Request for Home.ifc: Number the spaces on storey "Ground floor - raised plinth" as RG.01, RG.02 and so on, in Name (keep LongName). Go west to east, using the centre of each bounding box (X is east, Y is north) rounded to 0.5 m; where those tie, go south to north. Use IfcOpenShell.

First a look at what the model holds.

```python
import ifcopenshell
import ifcopenshell.util.element
import ifcopenshell.util.placement

model = ifcopenshell.open("Home.ifc")
print(model.schema)
storey = next(s for s in model.by_type("IfcBuildingStorey") if s.Name == "Ground floor - raised plinth")
spaces = [e for e in ifcopenshell.util.element.get_decomposition(storey) if e.is_a("IfcSpace")]
for e in sorted(spaces, key=lambda e: e.id()):
    origin = ifcopenshell.util.placement.get_local_placement(e.ObjectPlacement)[:3, 3]
    print(e.id(), e.Name, e.LongName, origin.round(2) + 0.0, sep=" | ")
```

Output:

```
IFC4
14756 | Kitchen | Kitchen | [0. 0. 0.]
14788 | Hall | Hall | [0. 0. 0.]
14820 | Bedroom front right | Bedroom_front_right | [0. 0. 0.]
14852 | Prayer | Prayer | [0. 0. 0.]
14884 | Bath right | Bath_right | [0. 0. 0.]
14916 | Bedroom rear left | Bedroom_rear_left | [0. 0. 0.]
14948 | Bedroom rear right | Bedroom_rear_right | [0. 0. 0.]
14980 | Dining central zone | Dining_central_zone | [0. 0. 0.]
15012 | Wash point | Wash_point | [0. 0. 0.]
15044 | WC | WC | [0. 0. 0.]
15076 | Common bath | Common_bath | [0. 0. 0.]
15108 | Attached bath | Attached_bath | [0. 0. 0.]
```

```python
import ifcopenshell
import ifcopenshell.geom
import ifcopenshell.util.element
import ifcopenshell.util.shape

model = ifcopenshell.open("Home.ifc")
settings = ifcopenshell.geom.settings()
settings.set("use-world-coords", True)


def centre(element):
    shape = ifcopenshell.geom.create_shape(settings, element)
    return ifcopenshell.util.shape.get_bbox_centroid(shape.geometry)


storey = next(s for s in model.by_type("IfcBuildingStorey") if s.Name == "Ground floor - raised plinth")
spaces = [e for e in ifcopenshell.util.element.get_decomposition(storey) if e.is_a("IfcSpace")]

# Insertion points can sit at a corner or the storey origin, so sort by the geometry (in metres).
centres = {e: centre(e) for e in spaces}
spaces.sort(key=lambda e: (round(centres[e][0] / 0.5), centres[e][1]))

for i, e in enumerate(spaces, start=1):
    number = f"RG.{i:02d}"
    e.Name = number
    print(e.id(), number)

model.write("Home_edited.ifc")
```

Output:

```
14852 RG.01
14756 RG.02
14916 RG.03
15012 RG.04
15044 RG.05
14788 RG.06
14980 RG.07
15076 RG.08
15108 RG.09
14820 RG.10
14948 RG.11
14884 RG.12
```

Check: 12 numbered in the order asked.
